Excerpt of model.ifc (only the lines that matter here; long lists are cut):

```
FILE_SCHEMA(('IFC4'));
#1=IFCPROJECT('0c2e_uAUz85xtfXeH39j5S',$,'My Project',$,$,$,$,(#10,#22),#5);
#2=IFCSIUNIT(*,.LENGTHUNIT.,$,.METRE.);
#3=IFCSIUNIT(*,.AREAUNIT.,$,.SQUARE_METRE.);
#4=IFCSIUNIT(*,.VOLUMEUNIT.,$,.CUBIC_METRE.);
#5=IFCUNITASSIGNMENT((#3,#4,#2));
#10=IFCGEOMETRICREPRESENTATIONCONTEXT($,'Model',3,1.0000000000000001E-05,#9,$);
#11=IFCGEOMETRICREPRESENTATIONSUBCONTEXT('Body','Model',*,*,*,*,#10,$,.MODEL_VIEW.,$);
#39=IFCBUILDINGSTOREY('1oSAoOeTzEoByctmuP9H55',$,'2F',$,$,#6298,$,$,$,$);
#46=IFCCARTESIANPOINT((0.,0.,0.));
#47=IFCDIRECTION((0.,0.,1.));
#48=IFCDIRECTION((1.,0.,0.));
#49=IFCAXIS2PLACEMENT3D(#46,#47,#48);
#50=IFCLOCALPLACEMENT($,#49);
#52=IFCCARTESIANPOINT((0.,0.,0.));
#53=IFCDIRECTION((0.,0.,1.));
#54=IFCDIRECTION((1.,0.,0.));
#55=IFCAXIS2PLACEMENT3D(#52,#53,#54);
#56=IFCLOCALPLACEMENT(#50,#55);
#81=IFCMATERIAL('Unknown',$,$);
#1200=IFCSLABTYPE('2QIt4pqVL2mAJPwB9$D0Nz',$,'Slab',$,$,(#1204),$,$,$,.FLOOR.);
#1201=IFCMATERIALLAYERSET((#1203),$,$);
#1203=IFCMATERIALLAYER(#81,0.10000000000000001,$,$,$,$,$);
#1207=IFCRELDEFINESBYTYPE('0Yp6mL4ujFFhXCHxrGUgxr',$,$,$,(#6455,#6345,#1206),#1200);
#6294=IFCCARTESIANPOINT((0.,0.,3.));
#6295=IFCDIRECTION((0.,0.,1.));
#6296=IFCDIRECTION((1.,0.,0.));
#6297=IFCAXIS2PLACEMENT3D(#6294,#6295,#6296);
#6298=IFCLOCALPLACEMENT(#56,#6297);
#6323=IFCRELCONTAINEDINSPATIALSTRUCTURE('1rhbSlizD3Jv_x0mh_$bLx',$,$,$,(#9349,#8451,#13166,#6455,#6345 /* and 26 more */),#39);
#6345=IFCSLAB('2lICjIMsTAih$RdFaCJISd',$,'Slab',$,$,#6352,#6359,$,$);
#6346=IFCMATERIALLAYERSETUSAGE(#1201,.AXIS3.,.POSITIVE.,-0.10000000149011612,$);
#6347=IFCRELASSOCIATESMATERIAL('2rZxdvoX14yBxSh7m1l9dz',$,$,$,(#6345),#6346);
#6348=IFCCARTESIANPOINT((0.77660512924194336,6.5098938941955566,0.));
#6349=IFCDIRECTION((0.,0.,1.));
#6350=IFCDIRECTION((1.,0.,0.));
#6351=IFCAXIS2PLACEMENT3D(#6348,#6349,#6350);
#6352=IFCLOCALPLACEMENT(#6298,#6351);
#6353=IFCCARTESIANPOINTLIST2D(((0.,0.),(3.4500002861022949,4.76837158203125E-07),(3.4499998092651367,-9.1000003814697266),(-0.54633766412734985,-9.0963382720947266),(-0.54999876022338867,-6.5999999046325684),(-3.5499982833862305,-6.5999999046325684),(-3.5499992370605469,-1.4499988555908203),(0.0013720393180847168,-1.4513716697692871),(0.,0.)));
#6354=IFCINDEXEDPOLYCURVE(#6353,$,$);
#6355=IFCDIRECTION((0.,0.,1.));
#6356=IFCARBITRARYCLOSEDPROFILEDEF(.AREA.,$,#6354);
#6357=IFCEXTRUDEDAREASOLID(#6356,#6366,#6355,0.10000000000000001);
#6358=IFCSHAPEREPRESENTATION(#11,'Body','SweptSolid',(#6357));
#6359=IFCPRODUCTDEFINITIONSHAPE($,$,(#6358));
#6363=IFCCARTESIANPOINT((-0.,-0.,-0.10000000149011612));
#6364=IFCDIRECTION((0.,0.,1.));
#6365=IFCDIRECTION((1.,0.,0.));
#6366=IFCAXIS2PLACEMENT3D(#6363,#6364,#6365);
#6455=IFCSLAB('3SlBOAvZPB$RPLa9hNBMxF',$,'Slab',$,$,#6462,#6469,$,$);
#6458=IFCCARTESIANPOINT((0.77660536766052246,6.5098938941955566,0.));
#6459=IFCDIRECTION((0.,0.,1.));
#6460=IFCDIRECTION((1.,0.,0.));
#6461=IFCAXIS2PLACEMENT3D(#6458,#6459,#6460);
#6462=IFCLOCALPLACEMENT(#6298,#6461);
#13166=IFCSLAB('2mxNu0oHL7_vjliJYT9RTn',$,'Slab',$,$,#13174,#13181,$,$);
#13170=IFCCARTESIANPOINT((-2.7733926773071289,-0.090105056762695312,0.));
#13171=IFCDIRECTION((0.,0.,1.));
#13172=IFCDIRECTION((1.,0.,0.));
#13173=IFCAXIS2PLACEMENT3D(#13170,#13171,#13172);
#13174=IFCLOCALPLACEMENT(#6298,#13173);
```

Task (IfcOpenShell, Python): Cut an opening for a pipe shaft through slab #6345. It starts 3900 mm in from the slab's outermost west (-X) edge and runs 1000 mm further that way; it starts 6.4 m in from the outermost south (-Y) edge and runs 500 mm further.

```python
import numpy as np
import ifcopenshell
import ifcopenshell.api.feature
import ifcopenshell.api.geometry
import ifcopenshell.api.root
import ifcopenshell.geom
import ifcopenshell.util.placement
import ifcopenshell.util.representation
import ifcopenshell.util.shape
import ifcopenshell.util.unit

model = ifcopenshell.open("model.ifc")
unit_scale = ifcopenshell.util.unit.calculate_unit_scale(model)
settings = ifcopenshell.geom.settings()


def volume(element):
    """Net volume in cubic metres, openings subtracted."""
    shape = ifcopenshell.geom.create_shape(settings, element)
    return ifcopenshell.util.shape.get_volume(shape.geometry)


slab = model.by_id(6345)
before = volume(slab)

# Extent in the slab's own axes, in metres. The edges named are its -X and -Y sides.
slab_shape = ifcopenshell.geom.create_shape(settings, slab)
vertices = ifcopenshell.util.shape.get_vertices(slab_shape.geometry)
x_min, y_min, bottom = vertices.min(axis=0)
top = vertices[:, 2].max()

opening = ifcopenshell.api.root.create_entity(model, ifc_class="IfcOpeningElement", name="Pipe shaft opening", predefined_type="OPENING")
context = ifcopenshell.util.representation.get_context(model, "Model", "Body", "MODEL_VIEW")
width, depth = 1, 0.5
outline = [(0.0, 0.0), (width, 0.0), (width, depth), (0.0, depth), (0.0, 0.0)]
# Overshoot both faces by 50 mm so the cut is clean.
shape = ifcopenshell.api.geometry.add_slab_representation(
    model, context=context, depth=top - bottom + 0.1, polyline=outline
)
ifcopenshell.api.geometry.assign_representation(model, product=opening, representation=shape)

matrix = ifcopenshell.util.placement.get_local_placement(slab.ObjectPlacement)
matrix[:, 3] = matrix @ np.append(np.array([x_min + 3.9, y_min + 6.4, bottom - 0.05]) / unit_scale, 1.0)
ifcopenshell.api.geometry.edit_object_placement(model, product=opening, matrix=matrix, is_si=False)
ifcopenshell.api.feature.add_feature(model, feature=opening, element=slab)

after = volume(slab)

print(f"slab volume {before:.3f} -> {after:.3f} m3")

model.write("model_edited.ifc")
```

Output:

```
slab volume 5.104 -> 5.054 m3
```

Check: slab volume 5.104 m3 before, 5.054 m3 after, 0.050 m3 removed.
